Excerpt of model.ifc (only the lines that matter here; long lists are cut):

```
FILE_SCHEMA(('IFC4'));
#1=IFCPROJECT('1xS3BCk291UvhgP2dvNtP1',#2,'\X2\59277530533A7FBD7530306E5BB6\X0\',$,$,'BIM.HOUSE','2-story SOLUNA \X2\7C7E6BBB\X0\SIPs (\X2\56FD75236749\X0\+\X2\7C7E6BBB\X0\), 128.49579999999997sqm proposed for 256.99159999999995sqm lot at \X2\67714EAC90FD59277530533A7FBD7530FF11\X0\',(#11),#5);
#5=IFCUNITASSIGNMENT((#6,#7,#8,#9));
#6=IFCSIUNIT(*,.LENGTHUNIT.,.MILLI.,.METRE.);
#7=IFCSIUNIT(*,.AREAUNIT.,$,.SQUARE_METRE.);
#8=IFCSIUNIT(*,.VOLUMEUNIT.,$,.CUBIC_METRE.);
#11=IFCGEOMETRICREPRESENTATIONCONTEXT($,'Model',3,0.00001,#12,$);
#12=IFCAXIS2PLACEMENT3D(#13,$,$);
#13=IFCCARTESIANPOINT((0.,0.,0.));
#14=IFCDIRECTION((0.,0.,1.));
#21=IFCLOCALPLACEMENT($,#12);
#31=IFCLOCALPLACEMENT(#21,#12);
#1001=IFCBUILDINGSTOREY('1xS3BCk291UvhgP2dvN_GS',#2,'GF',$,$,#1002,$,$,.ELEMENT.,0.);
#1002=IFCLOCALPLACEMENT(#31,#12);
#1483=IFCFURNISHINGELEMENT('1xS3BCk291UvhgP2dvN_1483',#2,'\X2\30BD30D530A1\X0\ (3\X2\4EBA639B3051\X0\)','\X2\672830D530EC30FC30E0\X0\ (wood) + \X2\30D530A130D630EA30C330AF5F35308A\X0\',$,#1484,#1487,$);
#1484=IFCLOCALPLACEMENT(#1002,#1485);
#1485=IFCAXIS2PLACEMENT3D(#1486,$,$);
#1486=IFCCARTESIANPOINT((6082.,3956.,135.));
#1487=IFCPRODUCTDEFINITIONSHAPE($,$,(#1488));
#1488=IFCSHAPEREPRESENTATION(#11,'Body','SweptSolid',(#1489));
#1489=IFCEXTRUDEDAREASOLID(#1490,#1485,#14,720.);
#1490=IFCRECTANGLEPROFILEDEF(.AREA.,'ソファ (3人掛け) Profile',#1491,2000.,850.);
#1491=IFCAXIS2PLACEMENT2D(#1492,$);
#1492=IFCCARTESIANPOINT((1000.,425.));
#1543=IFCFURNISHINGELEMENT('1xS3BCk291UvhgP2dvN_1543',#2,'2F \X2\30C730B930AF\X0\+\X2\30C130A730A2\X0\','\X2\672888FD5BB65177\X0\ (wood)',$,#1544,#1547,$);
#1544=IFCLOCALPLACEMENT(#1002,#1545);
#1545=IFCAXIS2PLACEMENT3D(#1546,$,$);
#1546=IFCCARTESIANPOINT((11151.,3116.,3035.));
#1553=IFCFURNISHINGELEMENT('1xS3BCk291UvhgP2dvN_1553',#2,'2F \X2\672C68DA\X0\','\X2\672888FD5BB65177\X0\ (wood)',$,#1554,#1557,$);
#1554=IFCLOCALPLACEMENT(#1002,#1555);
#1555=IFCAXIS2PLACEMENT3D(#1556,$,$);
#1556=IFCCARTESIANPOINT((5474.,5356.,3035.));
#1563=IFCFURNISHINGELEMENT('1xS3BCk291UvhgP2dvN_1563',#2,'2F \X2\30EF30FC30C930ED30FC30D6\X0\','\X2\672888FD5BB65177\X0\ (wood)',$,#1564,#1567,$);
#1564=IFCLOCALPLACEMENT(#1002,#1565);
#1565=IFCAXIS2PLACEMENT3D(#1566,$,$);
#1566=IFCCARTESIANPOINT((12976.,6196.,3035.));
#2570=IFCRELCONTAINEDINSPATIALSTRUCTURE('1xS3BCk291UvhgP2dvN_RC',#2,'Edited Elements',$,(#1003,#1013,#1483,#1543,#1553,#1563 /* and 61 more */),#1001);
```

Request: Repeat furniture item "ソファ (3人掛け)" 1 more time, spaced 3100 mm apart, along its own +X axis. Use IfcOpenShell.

```python
import ifcopenshell
import ifcopenshell.api.geometry
import ifcopenshell.api.root
import ifcopenshell.util.element
import ifcopenshell.util.placement
import ifcopenshell.util.unit

model = ifcopenshell.open("model.ifc")
unit_scale = ifcopenshell.util.unit.calculate_unit_scale(model)


def reuse_history(source, copy):
    """copy_class also copies each property set's owner history, people and application; keep the originals."""
    for rel in copy.IsDefinedBy:
        if rel.is_a("IfcRelDefinesByProperties") and (history := rel.RelatingPropertyDefinition.OwnerHistory):
            rel.RelatingPropertyDefinition.OwnerHistory = source.OwnerHistory
            ifcopenshell.util.element.remove_deep2(model, history)


source = model.by_id(1483)
base = ifcopenshell.util.placement.get_local_placement(source.ObjectPlacement)
step = base[:3, 0] * 3.1 / unit_scale

for i in range(1, 2):
    copy = ifcopenshell.api.root.copy_class(model, product=source)
    copy.Representation = ifcopenshell.util.element.copy_deep(
        model, source.Representation, exclude=["IfcGeometricRepresentationContext", "IfcRepresentationMap"]
    )
    reuse_history(source, copy)
    matrix = base.copy()
    matrix[:3, 3] += i * step
    print("added at", matrix[:3, 3].round(3) + 0.0)
    ifcopenshell.api.geometry.edit_object_placement(model, product=copy, matrix=matrix, is_si=False)

model.write("model_v2.ifc")
```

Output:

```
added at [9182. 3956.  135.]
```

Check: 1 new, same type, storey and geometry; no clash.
